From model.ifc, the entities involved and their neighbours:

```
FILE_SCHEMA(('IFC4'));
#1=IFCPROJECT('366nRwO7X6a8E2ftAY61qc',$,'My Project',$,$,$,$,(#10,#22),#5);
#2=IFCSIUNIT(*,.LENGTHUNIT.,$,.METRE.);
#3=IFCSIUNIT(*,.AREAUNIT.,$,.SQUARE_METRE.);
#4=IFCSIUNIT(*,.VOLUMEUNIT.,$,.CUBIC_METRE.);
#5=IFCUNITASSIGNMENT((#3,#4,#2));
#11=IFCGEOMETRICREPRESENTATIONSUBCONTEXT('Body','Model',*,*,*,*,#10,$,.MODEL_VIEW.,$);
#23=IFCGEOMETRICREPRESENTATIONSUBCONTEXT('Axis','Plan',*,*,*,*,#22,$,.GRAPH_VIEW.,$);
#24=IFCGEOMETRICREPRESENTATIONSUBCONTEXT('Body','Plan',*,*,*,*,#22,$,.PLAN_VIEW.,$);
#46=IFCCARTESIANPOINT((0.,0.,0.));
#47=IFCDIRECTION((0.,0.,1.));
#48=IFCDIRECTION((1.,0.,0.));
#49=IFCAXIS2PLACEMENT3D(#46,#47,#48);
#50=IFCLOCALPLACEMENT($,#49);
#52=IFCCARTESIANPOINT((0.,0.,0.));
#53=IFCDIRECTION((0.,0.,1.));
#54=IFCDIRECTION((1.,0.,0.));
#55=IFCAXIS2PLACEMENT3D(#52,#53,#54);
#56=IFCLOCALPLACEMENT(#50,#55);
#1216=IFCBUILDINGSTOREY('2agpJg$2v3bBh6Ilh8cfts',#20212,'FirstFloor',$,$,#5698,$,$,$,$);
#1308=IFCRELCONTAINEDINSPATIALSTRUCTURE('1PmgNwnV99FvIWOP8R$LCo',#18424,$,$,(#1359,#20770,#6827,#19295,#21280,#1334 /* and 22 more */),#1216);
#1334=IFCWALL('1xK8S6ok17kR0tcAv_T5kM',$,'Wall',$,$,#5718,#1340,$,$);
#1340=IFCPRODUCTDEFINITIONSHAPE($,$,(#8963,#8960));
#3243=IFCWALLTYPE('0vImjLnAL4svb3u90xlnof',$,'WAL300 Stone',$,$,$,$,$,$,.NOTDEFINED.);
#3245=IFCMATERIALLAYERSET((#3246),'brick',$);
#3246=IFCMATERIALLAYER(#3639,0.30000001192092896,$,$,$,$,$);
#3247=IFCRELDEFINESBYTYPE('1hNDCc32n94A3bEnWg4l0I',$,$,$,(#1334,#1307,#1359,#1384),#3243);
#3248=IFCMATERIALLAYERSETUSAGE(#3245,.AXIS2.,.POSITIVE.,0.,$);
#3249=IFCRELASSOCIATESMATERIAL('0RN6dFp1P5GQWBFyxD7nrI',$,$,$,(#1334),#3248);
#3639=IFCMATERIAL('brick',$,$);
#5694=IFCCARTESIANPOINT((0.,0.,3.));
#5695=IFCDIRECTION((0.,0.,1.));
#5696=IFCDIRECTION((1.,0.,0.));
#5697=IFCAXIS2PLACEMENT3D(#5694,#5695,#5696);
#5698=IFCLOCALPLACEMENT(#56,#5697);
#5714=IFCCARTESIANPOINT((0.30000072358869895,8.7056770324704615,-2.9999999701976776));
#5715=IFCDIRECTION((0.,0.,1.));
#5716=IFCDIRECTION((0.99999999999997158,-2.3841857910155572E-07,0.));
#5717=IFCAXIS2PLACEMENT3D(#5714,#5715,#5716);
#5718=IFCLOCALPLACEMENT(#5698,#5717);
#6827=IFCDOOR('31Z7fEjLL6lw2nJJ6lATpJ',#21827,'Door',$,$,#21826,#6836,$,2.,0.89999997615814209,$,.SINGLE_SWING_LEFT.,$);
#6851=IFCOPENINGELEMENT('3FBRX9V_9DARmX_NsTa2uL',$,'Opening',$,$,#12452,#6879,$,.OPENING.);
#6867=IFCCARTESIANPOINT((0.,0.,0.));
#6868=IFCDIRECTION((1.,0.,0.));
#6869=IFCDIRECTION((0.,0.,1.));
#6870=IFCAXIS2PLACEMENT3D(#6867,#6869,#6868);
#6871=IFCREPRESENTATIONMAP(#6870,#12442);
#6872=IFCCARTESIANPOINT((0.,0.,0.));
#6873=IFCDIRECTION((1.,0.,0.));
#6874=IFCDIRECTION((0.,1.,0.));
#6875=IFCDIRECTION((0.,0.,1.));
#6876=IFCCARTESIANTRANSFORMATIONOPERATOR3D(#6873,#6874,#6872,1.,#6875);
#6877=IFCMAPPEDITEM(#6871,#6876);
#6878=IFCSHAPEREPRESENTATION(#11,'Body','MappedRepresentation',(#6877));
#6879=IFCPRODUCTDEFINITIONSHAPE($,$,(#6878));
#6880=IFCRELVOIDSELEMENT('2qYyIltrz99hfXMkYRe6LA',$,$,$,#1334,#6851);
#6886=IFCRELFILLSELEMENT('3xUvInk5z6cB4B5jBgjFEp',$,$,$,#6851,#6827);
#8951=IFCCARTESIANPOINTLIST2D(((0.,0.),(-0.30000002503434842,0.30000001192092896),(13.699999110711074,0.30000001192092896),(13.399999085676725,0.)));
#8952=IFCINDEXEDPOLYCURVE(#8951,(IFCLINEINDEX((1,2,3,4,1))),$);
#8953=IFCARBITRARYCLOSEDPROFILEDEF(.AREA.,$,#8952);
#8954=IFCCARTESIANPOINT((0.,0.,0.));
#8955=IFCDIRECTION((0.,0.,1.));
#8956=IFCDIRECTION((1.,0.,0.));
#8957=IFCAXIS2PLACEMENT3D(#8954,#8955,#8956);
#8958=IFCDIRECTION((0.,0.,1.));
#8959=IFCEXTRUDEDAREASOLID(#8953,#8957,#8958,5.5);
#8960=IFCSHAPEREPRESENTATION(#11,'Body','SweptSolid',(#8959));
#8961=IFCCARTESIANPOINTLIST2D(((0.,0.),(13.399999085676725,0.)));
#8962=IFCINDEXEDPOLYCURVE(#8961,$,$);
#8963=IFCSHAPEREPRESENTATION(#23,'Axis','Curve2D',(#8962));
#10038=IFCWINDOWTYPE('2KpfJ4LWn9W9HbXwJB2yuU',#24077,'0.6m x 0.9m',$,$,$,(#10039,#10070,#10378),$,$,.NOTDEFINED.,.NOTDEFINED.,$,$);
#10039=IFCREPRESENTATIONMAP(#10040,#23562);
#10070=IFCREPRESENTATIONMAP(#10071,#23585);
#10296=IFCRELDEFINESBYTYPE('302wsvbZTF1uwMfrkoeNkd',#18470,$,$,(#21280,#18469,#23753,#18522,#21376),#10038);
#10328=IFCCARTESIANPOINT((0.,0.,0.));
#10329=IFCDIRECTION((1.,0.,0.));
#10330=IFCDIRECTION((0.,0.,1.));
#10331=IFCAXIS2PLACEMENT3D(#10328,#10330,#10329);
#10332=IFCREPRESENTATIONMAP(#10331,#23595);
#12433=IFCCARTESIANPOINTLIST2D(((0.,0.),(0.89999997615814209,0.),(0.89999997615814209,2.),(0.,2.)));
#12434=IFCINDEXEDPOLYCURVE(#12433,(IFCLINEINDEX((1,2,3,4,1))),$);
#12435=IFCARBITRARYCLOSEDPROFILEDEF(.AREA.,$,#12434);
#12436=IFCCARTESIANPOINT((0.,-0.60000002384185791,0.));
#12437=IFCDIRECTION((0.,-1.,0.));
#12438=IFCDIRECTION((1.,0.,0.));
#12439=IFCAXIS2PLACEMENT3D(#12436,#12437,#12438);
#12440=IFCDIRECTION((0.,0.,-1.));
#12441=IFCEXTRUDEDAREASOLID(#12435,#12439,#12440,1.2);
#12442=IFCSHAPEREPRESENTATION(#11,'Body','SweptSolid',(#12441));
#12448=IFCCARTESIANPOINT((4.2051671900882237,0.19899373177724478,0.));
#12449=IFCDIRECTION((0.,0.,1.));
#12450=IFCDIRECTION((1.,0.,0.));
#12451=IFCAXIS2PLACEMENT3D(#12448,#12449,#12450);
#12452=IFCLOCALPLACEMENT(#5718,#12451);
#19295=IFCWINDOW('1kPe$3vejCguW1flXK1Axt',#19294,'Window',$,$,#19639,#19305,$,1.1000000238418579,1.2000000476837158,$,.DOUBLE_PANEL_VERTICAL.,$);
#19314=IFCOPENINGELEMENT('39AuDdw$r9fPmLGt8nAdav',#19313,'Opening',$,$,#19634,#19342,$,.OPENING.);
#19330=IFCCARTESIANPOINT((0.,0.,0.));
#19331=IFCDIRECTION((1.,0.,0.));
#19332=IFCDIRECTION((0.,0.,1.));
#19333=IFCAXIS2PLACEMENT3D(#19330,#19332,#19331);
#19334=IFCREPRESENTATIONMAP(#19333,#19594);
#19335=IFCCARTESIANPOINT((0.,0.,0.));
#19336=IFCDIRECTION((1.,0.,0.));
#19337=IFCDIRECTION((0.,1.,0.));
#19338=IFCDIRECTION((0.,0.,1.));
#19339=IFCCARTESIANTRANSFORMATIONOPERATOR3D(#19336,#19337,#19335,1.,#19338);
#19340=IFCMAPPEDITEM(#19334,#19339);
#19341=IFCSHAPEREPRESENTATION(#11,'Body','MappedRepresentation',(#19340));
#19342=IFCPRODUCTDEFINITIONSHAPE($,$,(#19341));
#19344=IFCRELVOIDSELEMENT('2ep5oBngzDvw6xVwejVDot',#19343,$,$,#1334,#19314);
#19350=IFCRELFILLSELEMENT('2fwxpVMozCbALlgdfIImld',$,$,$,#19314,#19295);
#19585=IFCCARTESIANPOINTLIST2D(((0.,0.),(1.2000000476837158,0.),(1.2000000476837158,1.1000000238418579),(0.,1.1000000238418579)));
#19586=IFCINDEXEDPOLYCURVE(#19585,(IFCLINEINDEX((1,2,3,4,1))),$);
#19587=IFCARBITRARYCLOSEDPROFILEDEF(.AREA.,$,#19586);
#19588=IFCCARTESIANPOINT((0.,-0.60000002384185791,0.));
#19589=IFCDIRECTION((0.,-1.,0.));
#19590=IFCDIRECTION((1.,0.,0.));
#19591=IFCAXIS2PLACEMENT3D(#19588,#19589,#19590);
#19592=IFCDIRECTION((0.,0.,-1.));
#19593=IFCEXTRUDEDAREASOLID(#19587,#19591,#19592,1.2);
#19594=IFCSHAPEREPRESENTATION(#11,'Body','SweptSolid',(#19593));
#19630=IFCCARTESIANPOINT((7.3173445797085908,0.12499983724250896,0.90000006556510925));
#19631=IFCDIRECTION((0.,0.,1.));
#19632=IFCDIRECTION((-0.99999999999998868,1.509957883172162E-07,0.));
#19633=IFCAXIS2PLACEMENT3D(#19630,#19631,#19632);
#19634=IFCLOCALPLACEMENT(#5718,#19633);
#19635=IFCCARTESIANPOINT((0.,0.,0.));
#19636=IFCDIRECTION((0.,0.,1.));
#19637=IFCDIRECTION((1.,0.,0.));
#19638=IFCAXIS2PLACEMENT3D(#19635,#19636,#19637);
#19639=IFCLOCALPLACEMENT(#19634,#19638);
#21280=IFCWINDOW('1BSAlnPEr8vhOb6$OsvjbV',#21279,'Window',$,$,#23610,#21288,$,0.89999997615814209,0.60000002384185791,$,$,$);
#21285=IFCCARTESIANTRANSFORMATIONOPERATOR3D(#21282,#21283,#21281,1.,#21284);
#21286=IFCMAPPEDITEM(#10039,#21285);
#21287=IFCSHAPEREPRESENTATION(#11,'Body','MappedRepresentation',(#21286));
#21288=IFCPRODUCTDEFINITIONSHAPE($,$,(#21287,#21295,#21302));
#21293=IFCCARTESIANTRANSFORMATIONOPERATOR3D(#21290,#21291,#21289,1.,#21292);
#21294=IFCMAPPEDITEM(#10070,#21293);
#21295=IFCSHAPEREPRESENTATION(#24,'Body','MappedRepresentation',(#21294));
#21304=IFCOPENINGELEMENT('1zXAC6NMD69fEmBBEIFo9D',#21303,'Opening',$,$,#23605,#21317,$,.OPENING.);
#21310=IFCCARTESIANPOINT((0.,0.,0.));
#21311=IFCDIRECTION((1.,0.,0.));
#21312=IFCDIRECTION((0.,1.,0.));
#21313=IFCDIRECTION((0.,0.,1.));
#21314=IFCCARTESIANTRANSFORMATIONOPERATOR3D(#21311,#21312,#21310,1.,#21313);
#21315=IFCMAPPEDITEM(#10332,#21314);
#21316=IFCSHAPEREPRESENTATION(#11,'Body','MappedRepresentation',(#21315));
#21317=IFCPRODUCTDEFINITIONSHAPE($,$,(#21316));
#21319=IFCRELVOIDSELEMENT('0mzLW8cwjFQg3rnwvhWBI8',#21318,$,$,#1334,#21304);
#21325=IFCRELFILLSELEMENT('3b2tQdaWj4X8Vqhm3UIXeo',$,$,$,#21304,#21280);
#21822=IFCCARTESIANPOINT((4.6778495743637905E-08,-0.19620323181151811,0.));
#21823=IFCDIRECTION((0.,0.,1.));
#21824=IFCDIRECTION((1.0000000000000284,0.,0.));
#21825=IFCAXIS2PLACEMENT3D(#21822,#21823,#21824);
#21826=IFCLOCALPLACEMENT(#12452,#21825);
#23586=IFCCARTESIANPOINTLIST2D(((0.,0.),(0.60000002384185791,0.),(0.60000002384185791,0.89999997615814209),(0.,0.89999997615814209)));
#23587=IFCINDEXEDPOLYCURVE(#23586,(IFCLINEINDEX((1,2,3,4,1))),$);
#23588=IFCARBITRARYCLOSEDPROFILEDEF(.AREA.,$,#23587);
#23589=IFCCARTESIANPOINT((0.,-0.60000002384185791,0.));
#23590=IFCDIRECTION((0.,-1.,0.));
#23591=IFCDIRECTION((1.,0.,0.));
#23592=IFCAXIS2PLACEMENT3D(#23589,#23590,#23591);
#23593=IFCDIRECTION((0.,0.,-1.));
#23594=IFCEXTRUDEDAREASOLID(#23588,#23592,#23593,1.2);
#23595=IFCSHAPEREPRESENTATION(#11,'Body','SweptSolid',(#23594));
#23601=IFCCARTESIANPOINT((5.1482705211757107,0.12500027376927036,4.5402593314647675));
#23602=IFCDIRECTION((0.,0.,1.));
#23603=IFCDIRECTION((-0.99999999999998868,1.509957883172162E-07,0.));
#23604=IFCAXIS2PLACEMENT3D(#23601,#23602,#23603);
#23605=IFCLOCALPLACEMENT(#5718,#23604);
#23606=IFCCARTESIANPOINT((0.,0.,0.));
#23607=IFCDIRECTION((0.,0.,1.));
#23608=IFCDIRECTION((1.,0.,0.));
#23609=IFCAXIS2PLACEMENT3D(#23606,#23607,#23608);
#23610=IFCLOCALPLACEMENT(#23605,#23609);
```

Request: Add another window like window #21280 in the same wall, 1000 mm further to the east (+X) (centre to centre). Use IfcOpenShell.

```python
import ifcopenshell
import ifcopenshell.api.feature
import ifcopenshell.api.geometry
import ifcopenshell.api.root
import ifcopenshell.geom
import ifcopenshell.util.element
import ifcopenshell.util.placement
import ifcopenshell.util.shape
import ifcopenshell.util.unit

model = ifcopenshell.open("model.ifc")
unit_scale = ifcopenshell.util.unit.calculate_unit_scale(model)
settings = ifcopenshell.geom.settings()


def volume(element):
    """Net volume in cubic metres, openings subtracted."""
    shape = ifcopenshell.geom.create_shape(settings, element)
    return ifcopenshell.util.shape.get_volume(shape.geometry)


window = model.by_guid("1BSAlnPEr8vhOb6$OsvjbV")
opening = window.FillsVoids[0].RelatingOpeningElement
wall = opening.VoidsElements[0].RelatingBuildingElement
before = volume(wall)
shift = ifcopenshell.util.placement.get_local_placement(wall.ObjectPlacement)[:3, 0] * 1 / unit_scale

# copy_class copies the void relationship, type, container and properties, but no geometry.
new_opening = ifcopenshell.api.root.copy_class(model, product=opening)
new_opening.Representation = ifcopenshell.util.element.copy_deep(
    model, opening.Representation, exclude=["IfcGeometricRepresentationContext", "IfcRepresentationMap"]
)
new_window = ifcopenshell.api.root.copy_class(model, product=window)
new_window.Representation = ifcopenshell.util.element.copy_deep(
    model, window.Representation, exclude=["IfcGeometricRepresentationContext", "IfcRepresentationMap"]
)
ifcopenshell.api.feature.add_filling(model, opening=new_opening, element=new_window)

for old, new in ((opening, new_opening), (window, new_window)):
    matrix = ifcopenshell.util.placement.get_local_placement(old.ObjectPlacement)
    matrix[:3, 3] += shift
    ifcopenshell.api.geometry.edit_object_placement(model, product=new, matrix=matrix, is_si=False)

after = volume(wall)

print(f"wall volume {before:.3f} -> {after:.3f} m3")

model.write("model_rev.ifc")
```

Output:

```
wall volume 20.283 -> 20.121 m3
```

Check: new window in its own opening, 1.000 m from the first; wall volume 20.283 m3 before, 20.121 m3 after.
